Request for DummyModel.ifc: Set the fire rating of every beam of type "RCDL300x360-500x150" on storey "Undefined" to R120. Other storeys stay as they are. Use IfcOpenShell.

First a look at what the model holds.

```python
import ifcopenshell
import ifcopenshell.util.element

model = ifcopenshell.open("DummyModel.ifc")
print(model.schema)
storey = next(s for s in model.by_type("IfcBuildingStorey") if s.Name == "Undefined")
beams = [e for e in ifcopenshell.util.element.get_decomposition(storey) if e.is_a("IfcBeam")]
seen = {}
for e in beams:
    element_type = ifcopenshell.util.element.get_type(e)
    key = (element_type.Name if element_type != e and element_type else None, ifcopenshell.util.element.get_pset(e, "Pset_BeamCommon", "FireRating"))
    seen[key] = seen.get(key, 0) + 1
for (name, value), count in sorted(seen.items(), key=str):
    print(count, "x", name, "|", value)
```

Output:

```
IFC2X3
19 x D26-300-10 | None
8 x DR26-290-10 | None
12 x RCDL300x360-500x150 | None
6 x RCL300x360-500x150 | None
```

```python
import ifcopenshell
import ifcopenshell.api.pset
import ifcopenshell.util.element

model = ifcopenshell.open("DummyModel.ifc")

storey = next(s for s in model.by_type("IfcBuildingStorey") if s.Name == "Undefined")
beams = [e for e in ifcopenshell.util.element.get_decomposition(storey) if e.is_a("IfcBeam")]

count = 0
for e in beams:
    element_type = ifcopenshell.util.element.get_type(e)
    if element_type in (None, e) or element_type.Name != "RCDL300x360-500x150":
        continue
    found = ifcopenshell.util.element.get_pset(e, "Pset_BeamCommon", should_inherit=False)
    if found:
        pset = model.by_id(found["id"])
        if len(ifcopenshell.util.element.get_elements_by_pset(pset)) > 1:
            pset = ifcopenshell.api.pset.unshare_pset(model, products=[e], pset=pset)[0]
    else:
        pset = ifcopenshell.api.pset.add_pset(model, product=e, name="Pset_BeamCommon")
    ifcopenshell.api.pset.edit_pset(model, pset=pset, properties={"FireRating": "R120"})
    count += 1

print(count, "beams updated")

model.write("DummyModel-out.ifc")
```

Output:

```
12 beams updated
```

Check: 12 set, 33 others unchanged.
